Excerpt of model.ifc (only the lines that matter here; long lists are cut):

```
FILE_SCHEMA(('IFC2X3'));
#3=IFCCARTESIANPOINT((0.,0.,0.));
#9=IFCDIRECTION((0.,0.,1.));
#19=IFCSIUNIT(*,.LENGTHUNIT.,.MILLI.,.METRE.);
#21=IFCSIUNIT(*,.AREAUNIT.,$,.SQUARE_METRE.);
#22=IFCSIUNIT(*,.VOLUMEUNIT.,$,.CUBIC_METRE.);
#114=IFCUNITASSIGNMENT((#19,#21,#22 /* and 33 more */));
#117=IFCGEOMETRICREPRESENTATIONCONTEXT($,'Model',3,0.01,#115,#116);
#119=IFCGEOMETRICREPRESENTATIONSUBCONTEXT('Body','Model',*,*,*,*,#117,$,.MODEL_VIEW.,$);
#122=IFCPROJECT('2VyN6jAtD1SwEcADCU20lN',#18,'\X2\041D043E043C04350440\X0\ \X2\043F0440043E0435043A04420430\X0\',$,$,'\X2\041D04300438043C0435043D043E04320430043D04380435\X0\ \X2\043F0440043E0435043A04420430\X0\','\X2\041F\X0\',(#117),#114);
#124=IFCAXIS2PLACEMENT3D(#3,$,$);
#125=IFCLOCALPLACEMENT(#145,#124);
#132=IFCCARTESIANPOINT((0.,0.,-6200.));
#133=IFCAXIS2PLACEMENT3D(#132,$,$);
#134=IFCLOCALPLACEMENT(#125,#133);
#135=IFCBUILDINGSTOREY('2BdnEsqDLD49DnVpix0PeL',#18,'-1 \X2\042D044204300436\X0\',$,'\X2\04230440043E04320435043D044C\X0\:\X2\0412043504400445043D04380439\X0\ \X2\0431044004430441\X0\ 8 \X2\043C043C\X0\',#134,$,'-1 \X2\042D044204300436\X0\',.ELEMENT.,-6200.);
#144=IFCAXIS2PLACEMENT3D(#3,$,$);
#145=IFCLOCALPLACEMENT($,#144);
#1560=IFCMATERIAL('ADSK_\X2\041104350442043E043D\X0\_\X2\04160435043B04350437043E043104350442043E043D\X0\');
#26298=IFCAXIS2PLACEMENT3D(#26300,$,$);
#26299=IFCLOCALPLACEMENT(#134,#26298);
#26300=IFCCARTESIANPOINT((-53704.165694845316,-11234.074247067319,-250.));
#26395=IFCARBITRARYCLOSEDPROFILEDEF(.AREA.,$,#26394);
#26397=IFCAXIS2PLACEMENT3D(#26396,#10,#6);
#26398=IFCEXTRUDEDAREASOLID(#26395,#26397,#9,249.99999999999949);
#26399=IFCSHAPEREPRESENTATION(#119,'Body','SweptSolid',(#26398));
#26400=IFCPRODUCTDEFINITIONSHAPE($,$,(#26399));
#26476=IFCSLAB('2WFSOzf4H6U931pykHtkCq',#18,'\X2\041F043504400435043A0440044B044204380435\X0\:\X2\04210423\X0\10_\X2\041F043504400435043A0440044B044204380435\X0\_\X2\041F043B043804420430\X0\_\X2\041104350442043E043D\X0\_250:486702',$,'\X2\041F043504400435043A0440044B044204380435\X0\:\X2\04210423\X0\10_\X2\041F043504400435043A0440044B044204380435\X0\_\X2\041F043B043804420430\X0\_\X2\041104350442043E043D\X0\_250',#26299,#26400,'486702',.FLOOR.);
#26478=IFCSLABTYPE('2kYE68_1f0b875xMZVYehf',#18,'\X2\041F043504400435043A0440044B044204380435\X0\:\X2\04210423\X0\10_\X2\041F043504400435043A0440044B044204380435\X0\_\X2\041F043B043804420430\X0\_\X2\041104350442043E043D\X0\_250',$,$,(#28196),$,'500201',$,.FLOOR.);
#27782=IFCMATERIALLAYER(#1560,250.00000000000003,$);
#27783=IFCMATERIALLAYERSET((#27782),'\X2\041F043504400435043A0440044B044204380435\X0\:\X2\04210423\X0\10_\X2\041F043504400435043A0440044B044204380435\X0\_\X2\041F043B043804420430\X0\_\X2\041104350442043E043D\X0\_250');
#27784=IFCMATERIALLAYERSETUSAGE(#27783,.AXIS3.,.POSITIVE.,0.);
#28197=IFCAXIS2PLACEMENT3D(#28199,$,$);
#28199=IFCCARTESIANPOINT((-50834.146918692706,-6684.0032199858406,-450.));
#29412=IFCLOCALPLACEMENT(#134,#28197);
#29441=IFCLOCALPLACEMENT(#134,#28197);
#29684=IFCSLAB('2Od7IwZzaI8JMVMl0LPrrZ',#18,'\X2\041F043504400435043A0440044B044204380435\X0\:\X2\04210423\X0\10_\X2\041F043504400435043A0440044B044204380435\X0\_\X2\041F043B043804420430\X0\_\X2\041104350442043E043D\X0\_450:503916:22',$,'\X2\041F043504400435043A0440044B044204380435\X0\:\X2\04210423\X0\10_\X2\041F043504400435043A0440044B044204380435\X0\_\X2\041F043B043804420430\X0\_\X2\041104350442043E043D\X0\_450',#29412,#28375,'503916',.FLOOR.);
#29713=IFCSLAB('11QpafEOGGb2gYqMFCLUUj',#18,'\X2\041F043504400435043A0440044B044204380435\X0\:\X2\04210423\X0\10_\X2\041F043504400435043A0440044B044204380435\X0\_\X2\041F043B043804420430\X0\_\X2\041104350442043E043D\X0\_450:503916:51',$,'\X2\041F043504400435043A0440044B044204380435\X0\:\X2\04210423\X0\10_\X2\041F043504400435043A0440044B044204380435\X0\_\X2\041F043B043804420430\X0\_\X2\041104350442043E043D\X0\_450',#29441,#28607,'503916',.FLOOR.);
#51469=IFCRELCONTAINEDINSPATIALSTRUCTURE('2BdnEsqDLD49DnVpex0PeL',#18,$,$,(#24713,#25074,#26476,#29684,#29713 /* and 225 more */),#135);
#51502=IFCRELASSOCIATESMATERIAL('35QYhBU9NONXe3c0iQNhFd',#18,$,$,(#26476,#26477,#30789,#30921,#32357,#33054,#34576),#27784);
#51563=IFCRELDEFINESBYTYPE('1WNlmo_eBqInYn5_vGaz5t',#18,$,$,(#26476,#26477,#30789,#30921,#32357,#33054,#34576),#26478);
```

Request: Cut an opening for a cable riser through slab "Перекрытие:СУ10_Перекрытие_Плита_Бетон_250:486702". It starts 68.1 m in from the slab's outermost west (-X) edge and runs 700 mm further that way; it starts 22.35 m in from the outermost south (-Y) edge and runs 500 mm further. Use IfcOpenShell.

```python
import numpy as np
import ifcopenshell
import ifcopenshell.api.feature
import ifcopenshell.api.geometry
import ifcopenshell.api.root
import ifcopenshell.geom
import ifcopenshell.util.placement
import ifcopenshell.util.representation
import ifcopenshell.util.shape
import ifcopenshell.util.unit

model = ifcopenshell.open("model.ifc")
unit_scale = ifcopenshell.util.unit.calculate_unit_scale(model)
settings = ifcopenshell.geom.settings()


def volume(element):
    """Net volume in cubic metres, openings subtracted."""
    shape = ifcopenshell.geom.create_shape(settings, element)
    return ifcopenshell.util.shape.get_volume(shape.geometry)


slab = model.by_guid("2WFSOzf4H6U931pykHtkCq")
before = volume(slab)

# Extent in the slab's own axes, in metres. The edges named are its -X and -Y sides.
slab_shape = ifcopenshell.geom.create_shape(settings, slab)
vertices = ifcopenshell.util.shape.get_vertices(slab_shape.geometry)
x_min, y_min, bottom = vertices.min(axis=0)
top = vertices[:, 2].max()

opening = ifcopenshell.api.root.create_entity(model, ifc_class="IfcOpeningElement", name="Cable riser opening")
context = ifcopenshell.util.representation.get_context(model, "Model", "Body", "MODEL_VIEW")
width, depth = 0.7, 0.5
outline = [(0.0, 0.0), (width, 0.0), (width, depth), (0.0, depth), (0.0, 0.0)]
# Overshoot both faces by 50 mm so the cut is clean.
shape = ifcopenshell.api.geometry.add_slab_representation(
    model, context=context, depth=top - bottom + 0.1, polyline=outline
)
ifcopenshell.api.geometry.assign_representation(model, product=opening, representation=shape)

matrix = ifcopenshell.util.placement.get_local_placement(slab.ObjectPlacement)
matrix[:, 3] = matrix @ np.append(np.array([x_min + 68.1, y_min + 22.35, bottom - 0.05]) / unit_scale, 1.0)
ifcopenshell.api.geometry.edit_object_placement(model, product=opening, matrix=matrix, is_si=False)
ifcopenshell.api.feature.add_feature(model, feature=opening, element=slab)

after = volume(slab)

print(f"slab volume {before:.3f} -> {after:.3f} m3")

model.write("model_v2.ifc")
```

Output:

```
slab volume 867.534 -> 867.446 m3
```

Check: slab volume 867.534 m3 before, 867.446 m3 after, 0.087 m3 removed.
